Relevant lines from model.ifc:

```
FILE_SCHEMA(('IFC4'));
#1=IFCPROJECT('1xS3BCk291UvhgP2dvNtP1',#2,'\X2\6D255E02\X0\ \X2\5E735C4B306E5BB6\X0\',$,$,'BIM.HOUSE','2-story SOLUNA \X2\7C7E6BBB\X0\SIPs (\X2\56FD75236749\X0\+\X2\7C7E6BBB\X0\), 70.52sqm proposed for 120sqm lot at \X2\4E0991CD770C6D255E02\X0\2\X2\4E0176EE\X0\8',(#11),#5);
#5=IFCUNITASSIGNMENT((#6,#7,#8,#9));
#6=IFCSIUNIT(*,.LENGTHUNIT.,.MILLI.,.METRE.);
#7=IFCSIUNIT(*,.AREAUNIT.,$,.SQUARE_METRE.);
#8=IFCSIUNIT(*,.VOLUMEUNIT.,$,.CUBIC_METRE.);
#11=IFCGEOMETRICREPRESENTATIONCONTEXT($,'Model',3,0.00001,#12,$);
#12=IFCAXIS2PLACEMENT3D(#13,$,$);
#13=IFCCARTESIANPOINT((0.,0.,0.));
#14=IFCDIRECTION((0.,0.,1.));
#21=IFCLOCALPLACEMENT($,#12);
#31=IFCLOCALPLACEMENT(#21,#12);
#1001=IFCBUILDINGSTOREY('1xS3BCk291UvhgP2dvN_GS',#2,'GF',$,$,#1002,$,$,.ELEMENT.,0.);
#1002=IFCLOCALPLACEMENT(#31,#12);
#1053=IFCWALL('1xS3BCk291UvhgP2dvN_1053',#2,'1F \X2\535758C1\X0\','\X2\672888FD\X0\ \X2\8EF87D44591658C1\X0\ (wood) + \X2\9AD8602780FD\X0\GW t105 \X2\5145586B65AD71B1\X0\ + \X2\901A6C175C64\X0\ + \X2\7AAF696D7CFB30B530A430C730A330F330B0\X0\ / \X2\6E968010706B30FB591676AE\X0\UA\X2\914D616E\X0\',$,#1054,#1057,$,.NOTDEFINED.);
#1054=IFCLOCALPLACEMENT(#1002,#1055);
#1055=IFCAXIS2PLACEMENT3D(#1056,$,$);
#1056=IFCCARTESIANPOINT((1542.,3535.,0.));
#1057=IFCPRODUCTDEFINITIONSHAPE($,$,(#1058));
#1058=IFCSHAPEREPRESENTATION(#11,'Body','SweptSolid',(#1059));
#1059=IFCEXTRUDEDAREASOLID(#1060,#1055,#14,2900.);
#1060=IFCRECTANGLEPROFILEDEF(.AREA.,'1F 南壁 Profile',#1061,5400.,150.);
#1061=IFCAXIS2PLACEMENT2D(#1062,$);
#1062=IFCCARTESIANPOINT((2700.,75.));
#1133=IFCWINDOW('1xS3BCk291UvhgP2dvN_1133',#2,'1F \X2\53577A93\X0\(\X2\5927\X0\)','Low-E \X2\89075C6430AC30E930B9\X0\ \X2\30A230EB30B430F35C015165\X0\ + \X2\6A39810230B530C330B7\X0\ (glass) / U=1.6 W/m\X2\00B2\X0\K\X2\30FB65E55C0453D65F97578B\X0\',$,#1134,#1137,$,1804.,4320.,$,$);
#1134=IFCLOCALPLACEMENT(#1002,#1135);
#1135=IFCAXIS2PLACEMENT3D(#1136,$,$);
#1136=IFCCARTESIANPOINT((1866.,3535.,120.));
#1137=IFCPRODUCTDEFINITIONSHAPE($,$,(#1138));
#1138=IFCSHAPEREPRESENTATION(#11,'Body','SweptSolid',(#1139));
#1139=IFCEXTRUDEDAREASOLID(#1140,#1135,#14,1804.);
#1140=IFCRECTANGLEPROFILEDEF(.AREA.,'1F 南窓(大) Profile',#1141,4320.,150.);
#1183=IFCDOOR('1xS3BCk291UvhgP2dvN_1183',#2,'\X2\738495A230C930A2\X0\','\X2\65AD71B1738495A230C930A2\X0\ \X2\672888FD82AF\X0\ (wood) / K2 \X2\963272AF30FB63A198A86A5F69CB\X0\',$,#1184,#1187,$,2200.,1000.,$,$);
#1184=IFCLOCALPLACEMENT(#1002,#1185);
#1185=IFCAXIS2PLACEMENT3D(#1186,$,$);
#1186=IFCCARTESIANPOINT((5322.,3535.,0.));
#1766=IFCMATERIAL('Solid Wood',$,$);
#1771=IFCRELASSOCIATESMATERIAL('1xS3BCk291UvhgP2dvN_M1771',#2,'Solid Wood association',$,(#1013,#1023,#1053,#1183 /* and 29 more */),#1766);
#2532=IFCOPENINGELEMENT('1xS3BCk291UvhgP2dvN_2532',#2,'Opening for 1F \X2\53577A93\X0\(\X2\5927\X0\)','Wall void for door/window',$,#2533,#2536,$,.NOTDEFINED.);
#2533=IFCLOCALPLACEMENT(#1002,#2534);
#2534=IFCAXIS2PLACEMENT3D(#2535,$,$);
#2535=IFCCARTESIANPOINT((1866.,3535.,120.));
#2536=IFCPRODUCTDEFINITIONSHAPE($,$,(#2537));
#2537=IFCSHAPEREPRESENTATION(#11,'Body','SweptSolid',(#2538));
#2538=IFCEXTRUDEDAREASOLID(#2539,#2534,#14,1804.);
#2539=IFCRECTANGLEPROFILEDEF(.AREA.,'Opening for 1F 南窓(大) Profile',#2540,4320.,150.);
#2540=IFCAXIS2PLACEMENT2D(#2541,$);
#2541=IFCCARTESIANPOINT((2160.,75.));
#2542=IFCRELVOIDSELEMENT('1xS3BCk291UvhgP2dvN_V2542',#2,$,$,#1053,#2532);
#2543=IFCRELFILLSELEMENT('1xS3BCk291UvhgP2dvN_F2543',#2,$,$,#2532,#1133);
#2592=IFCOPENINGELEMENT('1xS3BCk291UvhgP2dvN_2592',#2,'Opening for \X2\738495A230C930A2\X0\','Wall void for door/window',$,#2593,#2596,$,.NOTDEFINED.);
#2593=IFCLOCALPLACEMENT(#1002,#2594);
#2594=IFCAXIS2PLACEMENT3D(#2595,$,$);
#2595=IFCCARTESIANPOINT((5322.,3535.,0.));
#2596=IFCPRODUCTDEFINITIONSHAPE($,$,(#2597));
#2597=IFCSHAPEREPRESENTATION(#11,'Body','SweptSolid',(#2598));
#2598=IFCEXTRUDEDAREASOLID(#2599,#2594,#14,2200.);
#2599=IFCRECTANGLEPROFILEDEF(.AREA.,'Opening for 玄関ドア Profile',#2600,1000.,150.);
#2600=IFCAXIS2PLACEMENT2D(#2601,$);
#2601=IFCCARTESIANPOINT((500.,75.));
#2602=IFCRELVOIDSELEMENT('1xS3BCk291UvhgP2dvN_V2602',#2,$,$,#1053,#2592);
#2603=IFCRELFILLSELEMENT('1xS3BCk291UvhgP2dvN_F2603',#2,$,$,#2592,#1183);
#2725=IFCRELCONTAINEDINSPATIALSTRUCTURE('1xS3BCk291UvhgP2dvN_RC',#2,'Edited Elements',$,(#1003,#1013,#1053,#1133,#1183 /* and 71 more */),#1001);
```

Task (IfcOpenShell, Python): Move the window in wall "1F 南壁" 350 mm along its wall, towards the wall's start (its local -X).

```python
import ifcopenshell
import ifcopenshell.api.geometry
import ifcopenshell.util.placement

model = ifcopenshell.open("model.ifc")

window = model.by_guid("1xS3BCk291UvhgP2dvN_1133")
opening = window.FillsVoids[0].RelatingOpeningElement
wall = opening.VoidsElements[0].RelatingBuildingElement

wall_matrix = ifcopenshell.util.placement.get_local_placement(wall.ObjectPlacement)
shift = wall_matrix[:3, 0] * -350.0
before = ifcopenshell.util.placement.get_local_placement(window.ObjectPlacement)[:3, 3].copy()

# The window is not placed relative to its opening, so move both.
for product in (opening, window):
    matrix = ifcopenshell.util.placement.get_local_placement(product.ObjectPlacement)
    matrix[:3, 3] += shift
    ifcopenshell.api.geometry.edit_object_placement(model, product=product, matrix=matrix, is_si=False)

after = ifcopenshell.util.placement.get_local_placement(window.ObjectPlacement)[:3, 3]
print("window moved by", (after - before).round(3) + 0.0)

model.write("model-out.ifc")
```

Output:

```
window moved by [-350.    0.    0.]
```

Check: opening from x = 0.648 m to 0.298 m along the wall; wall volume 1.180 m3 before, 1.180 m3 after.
